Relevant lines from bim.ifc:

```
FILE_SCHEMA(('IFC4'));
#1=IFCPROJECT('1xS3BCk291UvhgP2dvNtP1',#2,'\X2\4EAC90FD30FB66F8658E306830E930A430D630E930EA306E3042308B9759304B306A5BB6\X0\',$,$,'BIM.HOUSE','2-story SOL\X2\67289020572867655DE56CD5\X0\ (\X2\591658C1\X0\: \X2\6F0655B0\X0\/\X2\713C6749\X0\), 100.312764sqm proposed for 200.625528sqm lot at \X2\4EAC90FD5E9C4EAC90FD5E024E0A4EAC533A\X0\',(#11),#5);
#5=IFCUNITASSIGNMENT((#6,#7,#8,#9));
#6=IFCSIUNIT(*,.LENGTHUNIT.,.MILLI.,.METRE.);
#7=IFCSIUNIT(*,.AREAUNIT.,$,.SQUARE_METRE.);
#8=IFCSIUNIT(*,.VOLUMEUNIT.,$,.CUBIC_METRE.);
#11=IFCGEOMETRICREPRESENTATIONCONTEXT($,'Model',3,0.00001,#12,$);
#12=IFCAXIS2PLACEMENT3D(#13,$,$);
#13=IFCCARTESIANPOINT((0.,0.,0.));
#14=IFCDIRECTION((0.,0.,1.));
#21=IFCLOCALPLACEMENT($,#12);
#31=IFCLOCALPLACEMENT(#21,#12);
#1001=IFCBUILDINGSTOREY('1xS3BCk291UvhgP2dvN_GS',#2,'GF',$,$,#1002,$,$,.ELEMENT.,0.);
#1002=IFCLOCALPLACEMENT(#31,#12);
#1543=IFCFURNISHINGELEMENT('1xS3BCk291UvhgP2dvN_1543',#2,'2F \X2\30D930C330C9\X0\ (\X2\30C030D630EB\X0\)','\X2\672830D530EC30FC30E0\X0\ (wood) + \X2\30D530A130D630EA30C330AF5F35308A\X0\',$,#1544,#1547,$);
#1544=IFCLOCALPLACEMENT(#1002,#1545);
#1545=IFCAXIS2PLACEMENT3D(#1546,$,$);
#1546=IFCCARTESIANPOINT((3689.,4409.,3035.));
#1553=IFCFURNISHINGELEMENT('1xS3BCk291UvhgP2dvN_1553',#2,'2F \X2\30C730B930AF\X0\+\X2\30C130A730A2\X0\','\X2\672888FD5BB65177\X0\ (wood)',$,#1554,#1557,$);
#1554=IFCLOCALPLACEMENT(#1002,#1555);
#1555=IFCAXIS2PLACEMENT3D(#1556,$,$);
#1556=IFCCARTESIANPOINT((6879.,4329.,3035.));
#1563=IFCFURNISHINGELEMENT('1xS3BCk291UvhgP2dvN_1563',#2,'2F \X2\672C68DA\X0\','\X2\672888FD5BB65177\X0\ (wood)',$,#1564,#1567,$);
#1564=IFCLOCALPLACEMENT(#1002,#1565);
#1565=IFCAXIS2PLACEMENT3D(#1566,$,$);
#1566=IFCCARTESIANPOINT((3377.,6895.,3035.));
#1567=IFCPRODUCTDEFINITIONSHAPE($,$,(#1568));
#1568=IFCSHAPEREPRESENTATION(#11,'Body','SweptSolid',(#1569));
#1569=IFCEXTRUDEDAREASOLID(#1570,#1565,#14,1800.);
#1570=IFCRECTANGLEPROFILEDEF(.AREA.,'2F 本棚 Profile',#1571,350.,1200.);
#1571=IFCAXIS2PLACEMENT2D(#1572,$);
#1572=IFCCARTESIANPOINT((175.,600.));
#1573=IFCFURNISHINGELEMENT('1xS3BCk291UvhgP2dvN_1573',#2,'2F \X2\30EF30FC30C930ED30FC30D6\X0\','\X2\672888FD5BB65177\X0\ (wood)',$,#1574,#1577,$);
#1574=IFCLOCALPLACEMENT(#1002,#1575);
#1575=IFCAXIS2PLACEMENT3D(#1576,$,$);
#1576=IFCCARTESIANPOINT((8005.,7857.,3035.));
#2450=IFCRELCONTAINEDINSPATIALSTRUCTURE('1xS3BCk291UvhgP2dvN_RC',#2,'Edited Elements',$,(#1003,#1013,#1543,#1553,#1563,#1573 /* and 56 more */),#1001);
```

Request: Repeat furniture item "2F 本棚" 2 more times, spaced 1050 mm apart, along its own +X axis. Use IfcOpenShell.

```python
import ifcopenshell
import ifcopenshell.api.geometry
import ifcopenshell.api.root
import ifcopenshell.util.element
import ifcopenshell.util.placement
import ifcopenshell.util.unit

model = ifcopenshell.open("bim.ifc")
unit_scale = ifcopenshell.util.unit.calculate_unit_scale(model)


def reuse_history(source, copy):
    """copy_class also copies each property set's owner history, people and application; keep the originals."""
    for rel in copy.IsDefinedBy:
        if rel.is_a("IfcRelDefinesByProperties") and (history := rel.RelatingPropertyDefinition.OwnerHistory):
            rel.RelatingPropertyDefinition.OwnerHistory = source.OwnerHistory
            ifcopenshell.util.element.remove_deep2(model, history)


source = model.by_guid("1xS3BCk291UvhgP2dvN_1563")
base = ifcopenshell.util.placement.get_local_placement(source.ObjectPlacement)
step = base[:3, 0] * 1.05 / unit_scale

for i in range(1, 3):
    copy = ifcopenshell.api.root.copy_class(model, product=source)
    copy.Representation = ifcopenshell.util.element.copy_deep(
        model, source.Representation, exclude=["IfcGeometricRepresentationContext", "IfcRepresentationMap"]
    )
    reuse_history(source, copy)
    matrix = base.copy()
    matrix[:3, 3] += i * step
    print("added at", matrix[:3, 3].round(3) + 0.0)
    ifcopenshell.api.geometry.edit_object_placement(model, product=copy, matrix=matrix, is_si=False)

model.write("bim_updated.ifc")
```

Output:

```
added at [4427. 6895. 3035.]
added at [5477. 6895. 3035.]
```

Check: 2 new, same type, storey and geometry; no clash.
